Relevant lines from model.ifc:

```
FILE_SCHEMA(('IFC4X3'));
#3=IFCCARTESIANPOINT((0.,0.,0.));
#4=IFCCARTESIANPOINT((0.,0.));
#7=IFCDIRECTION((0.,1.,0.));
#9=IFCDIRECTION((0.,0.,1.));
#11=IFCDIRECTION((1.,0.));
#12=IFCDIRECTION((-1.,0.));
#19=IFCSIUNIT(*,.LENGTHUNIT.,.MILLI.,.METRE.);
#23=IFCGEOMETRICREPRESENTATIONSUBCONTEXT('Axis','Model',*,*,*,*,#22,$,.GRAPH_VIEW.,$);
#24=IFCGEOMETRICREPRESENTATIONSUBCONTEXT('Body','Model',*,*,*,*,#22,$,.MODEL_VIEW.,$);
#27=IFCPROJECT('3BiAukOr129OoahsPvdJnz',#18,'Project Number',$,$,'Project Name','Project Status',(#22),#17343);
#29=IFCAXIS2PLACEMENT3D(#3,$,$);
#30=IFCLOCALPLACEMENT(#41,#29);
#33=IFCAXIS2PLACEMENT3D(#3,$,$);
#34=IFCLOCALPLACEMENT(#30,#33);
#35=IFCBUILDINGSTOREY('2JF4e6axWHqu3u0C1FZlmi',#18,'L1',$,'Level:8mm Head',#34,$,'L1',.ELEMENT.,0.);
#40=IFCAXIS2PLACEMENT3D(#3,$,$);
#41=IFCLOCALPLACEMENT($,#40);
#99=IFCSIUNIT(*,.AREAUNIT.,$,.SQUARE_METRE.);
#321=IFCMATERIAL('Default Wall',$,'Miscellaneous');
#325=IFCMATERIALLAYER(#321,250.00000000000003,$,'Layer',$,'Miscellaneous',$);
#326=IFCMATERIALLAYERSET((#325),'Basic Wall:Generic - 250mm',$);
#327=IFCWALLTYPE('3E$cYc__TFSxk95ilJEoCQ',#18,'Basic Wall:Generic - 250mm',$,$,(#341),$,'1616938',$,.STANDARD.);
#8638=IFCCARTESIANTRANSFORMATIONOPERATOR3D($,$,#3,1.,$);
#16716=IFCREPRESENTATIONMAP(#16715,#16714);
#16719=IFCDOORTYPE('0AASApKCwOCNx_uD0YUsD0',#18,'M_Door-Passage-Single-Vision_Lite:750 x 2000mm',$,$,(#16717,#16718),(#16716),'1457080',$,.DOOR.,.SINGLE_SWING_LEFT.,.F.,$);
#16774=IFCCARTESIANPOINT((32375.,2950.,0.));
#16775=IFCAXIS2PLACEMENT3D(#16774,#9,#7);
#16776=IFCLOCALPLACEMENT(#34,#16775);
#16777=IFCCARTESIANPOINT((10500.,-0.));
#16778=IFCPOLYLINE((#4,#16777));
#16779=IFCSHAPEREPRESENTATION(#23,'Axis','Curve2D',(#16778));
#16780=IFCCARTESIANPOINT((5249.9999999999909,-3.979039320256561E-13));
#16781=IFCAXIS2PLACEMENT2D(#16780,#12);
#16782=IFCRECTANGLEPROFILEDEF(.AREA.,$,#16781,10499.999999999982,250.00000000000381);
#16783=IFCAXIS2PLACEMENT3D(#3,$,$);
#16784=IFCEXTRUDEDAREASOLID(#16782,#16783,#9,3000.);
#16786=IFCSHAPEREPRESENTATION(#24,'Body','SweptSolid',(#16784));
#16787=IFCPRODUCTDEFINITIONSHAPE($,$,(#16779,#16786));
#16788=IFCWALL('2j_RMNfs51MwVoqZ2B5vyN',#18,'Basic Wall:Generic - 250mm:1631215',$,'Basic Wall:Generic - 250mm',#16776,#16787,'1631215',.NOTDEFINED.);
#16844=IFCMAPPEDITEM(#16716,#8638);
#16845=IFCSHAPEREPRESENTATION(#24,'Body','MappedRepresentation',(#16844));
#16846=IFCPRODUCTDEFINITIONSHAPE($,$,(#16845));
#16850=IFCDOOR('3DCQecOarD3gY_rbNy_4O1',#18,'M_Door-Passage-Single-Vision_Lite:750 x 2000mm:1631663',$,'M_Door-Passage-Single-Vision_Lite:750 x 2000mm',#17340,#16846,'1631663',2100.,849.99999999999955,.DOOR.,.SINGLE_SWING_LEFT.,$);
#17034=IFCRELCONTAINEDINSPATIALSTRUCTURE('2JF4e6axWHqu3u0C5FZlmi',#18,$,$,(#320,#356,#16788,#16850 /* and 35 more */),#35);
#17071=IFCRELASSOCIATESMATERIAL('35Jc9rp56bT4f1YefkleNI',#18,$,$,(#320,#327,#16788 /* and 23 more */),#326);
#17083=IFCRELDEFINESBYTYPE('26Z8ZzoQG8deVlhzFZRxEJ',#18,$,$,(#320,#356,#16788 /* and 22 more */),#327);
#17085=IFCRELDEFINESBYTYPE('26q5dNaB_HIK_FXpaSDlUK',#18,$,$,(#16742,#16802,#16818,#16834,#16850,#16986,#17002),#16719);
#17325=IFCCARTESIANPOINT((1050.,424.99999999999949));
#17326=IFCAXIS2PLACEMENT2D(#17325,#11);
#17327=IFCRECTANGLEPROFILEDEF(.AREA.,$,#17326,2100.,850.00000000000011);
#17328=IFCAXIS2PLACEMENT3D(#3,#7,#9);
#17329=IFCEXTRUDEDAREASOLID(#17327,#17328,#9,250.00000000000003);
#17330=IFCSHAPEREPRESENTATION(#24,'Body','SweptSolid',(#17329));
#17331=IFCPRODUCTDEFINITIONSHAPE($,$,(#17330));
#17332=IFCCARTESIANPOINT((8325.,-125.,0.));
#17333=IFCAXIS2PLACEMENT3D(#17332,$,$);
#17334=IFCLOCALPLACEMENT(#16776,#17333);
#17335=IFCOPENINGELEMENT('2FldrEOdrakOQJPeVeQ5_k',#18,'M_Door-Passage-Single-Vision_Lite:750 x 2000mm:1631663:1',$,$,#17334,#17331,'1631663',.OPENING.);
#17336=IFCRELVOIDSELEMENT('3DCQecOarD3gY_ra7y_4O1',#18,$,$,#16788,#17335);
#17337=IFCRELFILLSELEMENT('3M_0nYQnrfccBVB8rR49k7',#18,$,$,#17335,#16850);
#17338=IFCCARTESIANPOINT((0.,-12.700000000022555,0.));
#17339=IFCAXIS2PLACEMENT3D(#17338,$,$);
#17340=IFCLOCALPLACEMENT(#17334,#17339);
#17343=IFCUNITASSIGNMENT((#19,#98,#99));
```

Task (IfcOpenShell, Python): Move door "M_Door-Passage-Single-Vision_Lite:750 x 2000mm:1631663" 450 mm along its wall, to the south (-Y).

```python
import ifcopenshell
import ifcopenshell.api.geometry
import ifcopenshell.util.placement
import ifcopenshell.util.unit

model = ifcopenshell.open("model.ifc")
unit_scale = ifcopenshell.util.unit.calculate_unit_scale(model)

door = model.by_id(16850)
opening = door.FillsVoids[0].RelatingOpeningElement
wall = opening.VoidsElements[0].RelatingBuildingElement

wall_matrix = ifcopenshell.util.placement.get_local_placement(wall.ObjectPlacement)
shift = wall_matrix[:3, 0] * -0.45 / unit_scale
before = ifcopenshell.util.placement.get_local_placement(door.ObjectPlacement)[:3, 3].copy()

# The door is placed relative to its opening, so it follows when the opening moves.
matrix = ifcopenshell.util.placement.get_local_placement(opening.ObjectPlacement)
matrix[:3, 3] += shift
ifcopenshell.api.geometry.edit_object_placement(
    model, product=opening, matrix=matrix, is_si=False, should_transform_children=True
)

after = ifcopenshell.util.placement.get_local_placement(door.ObjectPlacement)[:3, 3]
print("door moved by", (after - before).round(3) + 0.0)

model.write("model_updated.ifc")
```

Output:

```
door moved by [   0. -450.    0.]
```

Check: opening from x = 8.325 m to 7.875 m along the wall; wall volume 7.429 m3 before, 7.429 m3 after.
